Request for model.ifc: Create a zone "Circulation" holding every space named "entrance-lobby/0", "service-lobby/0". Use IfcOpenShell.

First a look at what the model holds.

```python
import ifcopenshell

model = ifcopenshell.open("model.ifc")
print(model.schema)
seen = {}
for space in model.by_type("IfcSpace"):
    seen[space.Name] = seen.get(space.Name, 0) + 1
for name, count in sorted(seen.items(), key=str):
    print(count, "x", name)
print("zones:", [z.Name for z in model.by_type("IfcZone")][:20])
```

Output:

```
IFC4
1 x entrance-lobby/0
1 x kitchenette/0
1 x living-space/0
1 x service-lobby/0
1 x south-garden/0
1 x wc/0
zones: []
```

```python
import ifcopenshell
import ifcopenshell.api.group
import ifcopenshell.api.root

model = ifcopenshell.open("model.ifc")

names = {"entrance-lobby/0", "service-lobby/0"}
spaces = [s for s in model.by_type("IfcSpace") if s.Name in names]

zone = ifcopenshell.api.root.create_entity(model, ifc_class="IfcZone", name="Circulation")
ifcopenshell.api.group.assign_group(model, products=spaces, group=zone)
print(len(spaces), "spaces in", zone.Name)

model.write("model-out.ifc")
```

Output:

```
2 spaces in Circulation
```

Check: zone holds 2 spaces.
